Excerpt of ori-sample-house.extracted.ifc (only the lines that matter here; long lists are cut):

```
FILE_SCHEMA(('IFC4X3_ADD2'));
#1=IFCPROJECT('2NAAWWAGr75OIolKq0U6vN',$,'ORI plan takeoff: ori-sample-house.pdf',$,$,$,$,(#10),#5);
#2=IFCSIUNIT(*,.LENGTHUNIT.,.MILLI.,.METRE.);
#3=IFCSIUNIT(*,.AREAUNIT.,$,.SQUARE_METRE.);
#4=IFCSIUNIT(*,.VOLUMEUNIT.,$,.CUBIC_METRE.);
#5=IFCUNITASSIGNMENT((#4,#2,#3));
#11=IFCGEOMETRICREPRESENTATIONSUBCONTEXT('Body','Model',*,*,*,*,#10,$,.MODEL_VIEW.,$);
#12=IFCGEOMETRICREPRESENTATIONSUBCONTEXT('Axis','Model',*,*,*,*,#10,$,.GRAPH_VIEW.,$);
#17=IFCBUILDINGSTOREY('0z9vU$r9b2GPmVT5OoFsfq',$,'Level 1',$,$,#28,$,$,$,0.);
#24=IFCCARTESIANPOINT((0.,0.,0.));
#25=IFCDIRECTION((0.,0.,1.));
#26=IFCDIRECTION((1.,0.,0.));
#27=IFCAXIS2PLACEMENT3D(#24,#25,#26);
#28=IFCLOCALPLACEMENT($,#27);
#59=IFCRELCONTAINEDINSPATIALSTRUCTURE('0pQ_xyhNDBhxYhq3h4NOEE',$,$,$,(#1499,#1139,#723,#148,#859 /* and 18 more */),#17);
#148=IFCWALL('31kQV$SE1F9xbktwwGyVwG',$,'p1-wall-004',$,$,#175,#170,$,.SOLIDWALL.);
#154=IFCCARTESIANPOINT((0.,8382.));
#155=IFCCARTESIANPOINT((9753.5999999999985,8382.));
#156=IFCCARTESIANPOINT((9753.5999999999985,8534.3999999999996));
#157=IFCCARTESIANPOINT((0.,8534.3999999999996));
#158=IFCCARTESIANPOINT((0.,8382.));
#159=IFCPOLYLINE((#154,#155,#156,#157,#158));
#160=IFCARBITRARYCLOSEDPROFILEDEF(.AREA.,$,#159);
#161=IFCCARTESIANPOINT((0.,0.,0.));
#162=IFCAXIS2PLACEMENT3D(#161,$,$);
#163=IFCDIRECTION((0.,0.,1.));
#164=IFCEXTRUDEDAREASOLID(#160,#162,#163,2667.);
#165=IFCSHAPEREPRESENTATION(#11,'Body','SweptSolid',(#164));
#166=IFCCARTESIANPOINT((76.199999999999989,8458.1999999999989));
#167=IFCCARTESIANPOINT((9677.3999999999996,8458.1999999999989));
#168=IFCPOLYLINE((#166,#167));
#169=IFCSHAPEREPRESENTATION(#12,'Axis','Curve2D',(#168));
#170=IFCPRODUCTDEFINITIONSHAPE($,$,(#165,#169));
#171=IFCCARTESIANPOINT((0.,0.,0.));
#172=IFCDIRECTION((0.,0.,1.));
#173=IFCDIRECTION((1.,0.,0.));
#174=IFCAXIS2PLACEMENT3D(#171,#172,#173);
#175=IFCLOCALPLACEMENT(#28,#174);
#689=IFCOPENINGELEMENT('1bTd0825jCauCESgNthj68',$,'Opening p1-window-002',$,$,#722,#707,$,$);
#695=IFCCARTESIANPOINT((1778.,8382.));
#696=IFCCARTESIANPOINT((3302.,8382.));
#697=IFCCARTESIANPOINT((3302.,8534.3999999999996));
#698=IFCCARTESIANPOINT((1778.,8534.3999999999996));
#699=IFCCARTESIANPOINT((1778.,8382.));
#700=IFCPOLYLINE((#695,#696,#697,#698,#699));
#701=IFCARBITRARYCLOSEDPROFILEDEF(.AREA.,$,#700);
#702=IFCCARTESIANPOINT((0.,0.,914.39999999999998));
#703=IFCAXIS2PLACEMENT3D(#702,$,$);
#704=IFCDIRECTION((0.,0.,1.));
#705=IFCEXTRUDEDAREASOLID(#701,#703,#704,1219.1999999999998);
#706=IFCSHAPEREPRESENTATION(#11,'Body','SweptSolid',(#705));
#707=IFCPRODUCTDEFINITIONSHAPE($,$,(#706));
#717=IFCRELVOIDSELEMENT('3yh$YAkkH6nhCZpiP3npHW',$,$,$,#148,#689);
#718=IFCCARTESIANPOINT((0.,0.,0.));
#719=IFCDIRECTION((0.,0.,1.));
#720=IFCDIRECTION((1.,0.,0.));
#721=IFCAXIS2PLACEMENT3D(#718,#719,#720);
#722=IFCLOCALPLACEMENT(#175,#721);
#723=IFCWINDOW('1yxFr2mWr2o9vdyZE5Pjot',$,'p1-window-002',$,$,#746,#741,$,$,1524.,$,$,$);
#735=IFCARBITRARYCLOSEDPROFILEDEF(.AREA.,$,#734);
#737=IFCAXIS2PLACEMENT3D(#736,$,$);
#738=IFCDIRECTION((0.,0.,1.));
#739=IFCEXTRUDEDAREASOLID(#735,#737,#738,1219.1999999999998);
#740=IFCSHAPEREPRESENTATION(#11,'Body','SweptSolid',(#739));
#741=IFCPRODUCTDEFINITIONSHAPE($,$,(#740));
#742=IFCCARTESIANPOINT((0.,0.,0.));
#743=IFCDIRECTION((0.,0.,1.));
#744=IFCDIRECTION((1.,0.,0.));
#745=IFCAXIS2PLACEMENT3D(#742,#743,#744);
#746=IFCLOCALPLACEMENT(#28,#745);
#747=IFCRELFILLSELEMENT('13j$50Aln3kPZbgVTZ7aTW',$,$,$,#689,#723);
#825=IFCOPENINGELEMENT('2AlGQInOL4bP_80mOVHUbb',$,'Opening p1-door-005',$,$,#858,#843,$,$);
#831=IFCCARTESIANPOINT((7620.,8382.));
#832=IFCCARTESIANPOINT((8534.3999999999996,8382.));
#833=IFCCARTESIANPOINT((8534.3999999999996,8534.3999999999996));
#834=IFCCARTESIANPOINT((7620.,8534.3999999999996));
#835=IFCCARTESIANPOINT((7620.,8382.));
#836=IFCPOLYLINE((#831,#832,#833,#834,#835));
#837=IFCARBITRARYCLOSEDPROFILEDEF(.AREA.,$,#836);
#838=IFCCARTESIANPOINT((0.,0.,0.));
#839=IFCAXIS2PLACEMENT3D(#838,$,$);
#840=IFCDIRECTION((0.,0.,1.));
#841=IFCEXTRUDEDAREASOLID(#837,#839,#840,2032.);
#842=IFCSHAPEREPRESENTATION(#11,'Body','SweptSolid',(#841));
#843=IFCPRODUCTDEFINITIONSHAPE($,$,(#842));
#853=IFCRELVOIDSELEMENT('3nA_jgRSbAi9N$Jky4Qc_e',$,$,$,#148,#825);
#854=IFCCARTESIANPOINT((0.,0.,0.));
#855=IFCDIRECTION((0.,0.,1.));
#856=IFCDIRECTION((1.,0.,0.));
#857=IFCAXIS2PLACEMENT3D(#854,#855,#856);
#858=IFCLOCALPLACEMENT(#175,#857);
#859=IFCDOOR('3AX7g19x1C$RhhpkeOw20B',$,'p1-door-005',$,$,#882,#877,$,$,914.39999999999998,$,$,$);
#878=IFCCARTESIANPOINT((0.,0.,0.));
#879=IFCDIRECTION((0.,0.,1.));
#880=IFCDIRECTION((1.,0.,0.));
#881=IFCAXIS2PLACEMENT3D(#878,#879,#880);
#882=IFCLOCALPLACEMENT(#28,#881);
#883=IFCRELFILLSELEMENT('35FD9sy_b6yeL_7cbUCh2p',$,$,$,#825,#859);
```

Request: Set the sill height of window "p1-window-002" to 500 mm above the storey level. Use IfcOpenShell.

```python
import numpy as np
import ifcopenshell
import ifcopenshell.api.geometry
import ifcopenshell.geom
import ifcopenshell.util.element
import ifcopenshell.util.placement
import ifcopenshell.util.shape
import ifcopenshell.util.unit

model = ifcopenshell.open("ori-sample-house.extracted.ifc")
unit_scale = ifcopenshell.util.unit.calculate_unit_scale(model)

window = model.by_id(723)
opening = window.FillsVoids[0].RelatingOpeningElement
storey = ifcopenshell.util.element.get_container(window, ifc_class="IfcBuildingStorey")
level = ifcopenshell.util.placement.get_local_placement(storey.ObjectPlacement)[2, 3]

# The opening's origin need not be at the sill, so measure its lowest point.
shape = ifcopenshell.geom.create_shape(ifcopenshell.geom.settings(), opening)
bottom = ifcopenshell.util.shape.get_shape_bottom_elevation(shape, shape.geometry) / unit_scale
dz = level + 500.0 - bottom

shift = np.array([0.0, 0.0, dz])
# The window is not placed relative to its opening, so move both.
for product in (opening, window):
    matrix = ifcopenshell.util.placement.get_local_placement(product.ObjectPlacement)
    matrix[:3, 3] += shift
    ifcopenshell.api.geometry.edit_object_placement(model, product=product, matrix=matrix, is_si=False)

print(f"moved by {dz * unit_scale:+.3f} m")

model.write("ori-sample-house.extracted_edited.ifc")
```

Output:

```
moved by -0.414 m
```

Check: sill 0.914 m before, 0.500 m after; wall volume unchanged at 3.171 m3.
